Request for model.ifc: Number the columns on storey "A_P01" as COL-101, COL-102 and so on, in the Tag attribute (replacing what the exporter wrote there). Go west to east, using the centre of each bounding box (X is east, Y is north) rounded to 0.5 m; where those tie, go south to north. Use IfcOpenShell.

First a look at what the model holds.

```python
import ifcopenshell
import ifcopenshell.util.element
import ifcopenshell.util.placement

model = ifcopenshell.open("model.ifc")
print(model.schema)
storey = next(s for s in model.by_type("IfcBuildingStorey") if s.Name == "A_P01")
columns = [e for e in ifcopenshell.util.element.get_decomposition(storey) if e.is_a("IfcColumn")]
for e in sorted(columns, key=lambda e: e.id()):
    origin = ifcopenshell.util.placement.get_local_placement(e.ObjectPlacement)[:3, 3]
    print(e.id(), e.Tag, e.Name, origin.round(2) + 0.0, sep=" | ")
```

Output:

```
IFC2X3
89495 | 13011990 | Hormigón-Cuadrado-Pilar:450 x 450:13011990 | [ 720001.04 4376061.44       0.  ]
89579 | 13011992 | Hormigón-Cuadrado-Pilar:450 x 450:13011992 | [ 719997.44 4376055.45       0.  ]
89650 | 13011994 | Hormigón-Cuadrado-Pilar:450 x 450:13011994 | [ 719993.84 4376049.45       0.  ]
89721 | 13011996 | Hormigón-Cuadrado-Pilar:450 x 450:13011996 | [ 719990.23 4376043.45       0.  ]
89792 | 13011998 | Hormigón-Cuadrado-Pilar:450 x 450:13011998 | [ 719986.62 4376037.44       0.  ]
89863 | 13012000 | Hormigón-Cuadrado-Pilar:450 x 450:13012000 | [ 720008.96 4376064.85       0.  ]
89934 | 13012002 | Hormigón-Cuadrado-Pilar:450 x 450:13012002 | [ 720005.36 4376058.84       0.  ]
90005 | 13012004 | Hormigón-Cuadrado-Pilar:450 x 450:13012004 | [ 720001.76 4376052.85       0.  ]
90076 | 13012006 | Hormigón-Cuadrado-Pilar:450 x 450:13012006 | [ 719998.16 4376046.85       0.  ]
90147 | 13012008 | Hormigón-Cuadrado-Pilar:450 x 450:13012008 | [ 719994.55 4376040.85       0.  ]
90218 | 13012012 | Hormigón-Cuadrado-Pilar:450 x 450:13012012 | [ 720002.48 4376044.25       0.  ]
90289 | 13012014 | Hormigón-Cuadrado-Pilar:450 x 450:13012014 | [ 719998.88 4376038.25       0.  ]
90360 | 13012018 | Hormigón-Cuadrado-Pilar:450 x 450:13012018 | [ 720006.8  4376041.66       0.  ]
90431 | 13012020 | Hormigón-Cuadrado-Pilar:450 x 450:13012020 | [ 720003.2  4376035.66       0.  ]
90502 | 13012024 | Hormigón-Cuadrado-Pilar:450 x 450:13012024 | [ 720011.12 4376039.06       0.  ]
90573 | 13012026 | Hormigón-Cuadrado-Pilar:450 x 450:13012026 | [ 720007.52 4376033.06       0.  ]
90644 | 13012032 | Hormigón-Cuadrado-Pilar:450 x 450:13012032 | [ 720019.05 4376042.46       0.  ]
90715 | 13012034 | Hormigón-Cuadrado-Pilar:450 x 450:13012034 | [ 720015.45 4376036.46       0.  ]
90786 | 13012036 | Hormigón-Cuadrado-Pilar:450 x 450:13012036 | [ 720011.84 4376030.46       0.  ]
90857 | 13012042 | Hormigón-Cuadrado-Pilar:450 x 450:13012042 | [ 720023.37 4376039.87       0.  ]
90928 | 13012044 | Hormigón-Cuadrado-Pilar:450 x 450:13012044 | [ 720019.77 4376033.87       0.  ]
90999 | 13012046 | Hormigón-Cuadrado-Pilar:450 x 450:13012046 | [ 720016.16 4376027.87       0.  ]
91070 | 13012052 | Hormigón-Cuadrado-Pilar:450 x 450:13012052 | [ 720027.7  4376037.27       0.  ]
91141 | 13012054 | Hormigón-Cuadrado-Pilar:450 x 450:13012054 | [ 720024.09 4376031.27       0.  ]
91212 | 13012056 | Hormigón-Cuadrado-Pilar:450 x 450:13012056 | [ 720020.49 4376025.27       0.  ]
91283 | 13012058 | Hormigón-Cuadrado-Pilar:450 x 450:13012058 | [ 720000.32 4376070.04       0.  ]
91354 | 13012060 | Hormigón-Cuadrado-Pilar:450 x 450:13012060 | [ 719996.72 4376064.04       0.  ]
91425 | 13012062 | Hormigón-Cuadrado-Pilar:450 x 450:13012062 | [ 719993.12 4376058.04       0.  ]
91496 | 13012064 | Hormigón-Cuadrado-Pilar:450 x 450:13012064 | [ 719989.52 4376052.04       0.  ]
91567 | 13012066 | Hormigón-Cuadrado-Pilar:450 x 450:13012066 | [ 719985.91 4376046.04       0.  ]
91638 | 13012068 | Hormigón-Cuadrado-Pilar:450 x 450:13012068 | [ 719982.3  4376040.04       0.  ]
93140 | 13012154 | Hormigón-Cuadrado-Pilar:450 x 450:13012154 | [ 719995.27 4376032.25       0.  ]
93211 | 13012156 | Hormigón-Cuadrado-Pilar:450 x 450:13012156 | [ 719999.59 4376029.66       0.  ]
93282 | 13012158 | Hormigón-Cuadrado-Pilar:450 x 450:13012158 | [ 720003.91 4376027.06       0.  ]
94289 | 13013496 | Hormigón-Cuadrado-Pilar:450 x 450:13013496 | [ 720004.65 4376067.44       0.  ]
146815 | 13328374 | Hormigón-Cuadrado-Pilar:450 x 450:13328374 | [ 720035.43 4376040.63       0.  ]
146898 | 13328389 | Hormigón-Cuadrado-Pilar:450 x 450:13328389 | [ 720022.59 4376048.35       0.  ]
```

```python
import ifcopenshell
import ifcopenshell.geom
import ifcopenshell.util.element
import ifcopenshell.util.shape

model = ifcopenshell.open("model.ifc")
settings = ifcopenshell.geom.settings()
settings.set("use-world-coords", True)


def centre(element):
    shape = ifcopenshell.geom.create_shape(settings, element)
    return ifcopenshell.util.shape.get_bbox_centroid(shape.geometry)


storey = next(s for s in model.by_type("IfcBuildingStorey") if s.Name == "A_P01")
columns = [e for e in ifcopenshell.util.element.get_decomposition(storey) if e.is_a("IfcColumn")]

# Insertion points can sit at a corner or the storey origin, so sort by the geometry (in metres).
centres = {e: centre(e) for e in columns}
columns.sort(key=lambda e: (round(centres[e][0] / 0.5), centres[e][1]))

for i, e in enumerate(columns, start=1):
    number = f"COL-1{i:02d}"
    e.Tag = number
    print(e.id(), number)

model.write("model_updated.ifc")
```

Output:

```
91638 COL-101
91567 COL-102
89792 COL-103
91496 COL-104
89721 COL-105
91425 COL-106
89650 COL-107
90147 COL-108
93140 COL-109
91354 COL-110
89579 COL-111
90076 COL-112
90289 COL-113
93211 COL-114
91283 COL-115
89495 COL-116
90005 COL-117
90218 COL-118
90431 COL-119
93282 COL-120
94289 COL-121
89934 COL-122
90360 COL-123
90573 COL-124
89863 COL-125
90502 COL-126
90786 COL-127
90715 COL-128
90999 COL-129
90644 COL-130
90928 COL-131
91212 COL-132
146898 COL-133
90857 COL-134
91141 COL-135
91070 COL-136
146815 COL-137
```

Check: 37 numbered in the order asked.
